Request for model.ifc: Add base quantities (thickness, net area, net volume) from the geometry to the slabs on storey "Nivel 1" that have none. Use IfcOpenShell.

First a look at what the model holds.

```python
import ifcopenshell
import ifcopenshell.util.element
import ifcopenshell.util.unit

model = ifcopenshell.open("model.ifc")
print(model.schema)
for unit_type in ("LENGTHUNIT", "AREAUNIT", "VOLUMEUNIT"):
    print(unit_type, ifcopenshell.util.unit.calculate_unit_scale(model, unit_type))
storey = next(s for s in model.by_type("IfcBuildingStorey") if s.Name == "Nivel 1")
slabs = [e for e in ifcopenshell.util.element.get_decomposition(storey) if e.is_a("IfcSlab")]
for e in sorted(slabs, key=lambda e: e.id()):
    print(e.id(), e.is_a(), e.Name, list(ifcopenshell.util.element.get_psets(e, qtos_only=True)), sep=" | ")
```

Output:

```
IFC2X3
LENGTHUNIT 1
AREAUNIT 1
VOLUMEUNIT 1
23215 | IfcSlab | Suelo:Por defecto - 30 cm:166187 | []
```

```python
import ifcopenshell
import ifcopenshell.api.pset
import ifcopenshell.geom
import ifcopenshell.util.element
import ifcopenshell.util.shape
import ifcopenshell.util.unit

model = ifcopenshell.open("model.ifc")
unit_scale = ifcopenshell.util.unit.calculate_unit_scale(model)
area_scale = ifcopenshell.util.unit.calculate_unit_scale(model, "AREAUNIT")
volume_scale = ifcopenshell.util.unit.calculate_unit_scale(model, "VOLUMEUNIT")
settings = ifcopenshell.geom.settings()

storey = next(s for s in model.by_type("IfcBuildingStorey") if s.Name == "Nivel 1")
slabs = [e for e in ifcopenshell.util.element.get_decomposition(storey) if e.is_a("IfcSlab")]

for e in sorted(slabs, key=lambda e: e.id()):
    if ifcopenshell.util.element.get_psets(e, qtos_only=True, should_inherit=False):
        continue
    # Geometry comes back in metres, in the element's own axes.
    shape = ifcopenshell.geom.create_shape(settings, e)
    values = {
        "Width": ifcopenshell.util.shape.get_z(shape.geometry) / unit_scale,
        "NetArea": ifcopenshell.util.shape.get_footprint_area(shape.geometry) / area_scale,
        "NetVolume": ifcopenshell.util.shape.get_volume(shape.geometry) / volume_scale,
    }
    qto = ifcopenshell.api.pset.add_qto(model, product=e, name="BaseQuantities")
    ifcopenshell.api.pset.edit_qto(model, qto=qto, properties=values)
    print(e.id(), {k: round(v, 3) for k, v in values.items()})

model.write("model_v2.ifc")
```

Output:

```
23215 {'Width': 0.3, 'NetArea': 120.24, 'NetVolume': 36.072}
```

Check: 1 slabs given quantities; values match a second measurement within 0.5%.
